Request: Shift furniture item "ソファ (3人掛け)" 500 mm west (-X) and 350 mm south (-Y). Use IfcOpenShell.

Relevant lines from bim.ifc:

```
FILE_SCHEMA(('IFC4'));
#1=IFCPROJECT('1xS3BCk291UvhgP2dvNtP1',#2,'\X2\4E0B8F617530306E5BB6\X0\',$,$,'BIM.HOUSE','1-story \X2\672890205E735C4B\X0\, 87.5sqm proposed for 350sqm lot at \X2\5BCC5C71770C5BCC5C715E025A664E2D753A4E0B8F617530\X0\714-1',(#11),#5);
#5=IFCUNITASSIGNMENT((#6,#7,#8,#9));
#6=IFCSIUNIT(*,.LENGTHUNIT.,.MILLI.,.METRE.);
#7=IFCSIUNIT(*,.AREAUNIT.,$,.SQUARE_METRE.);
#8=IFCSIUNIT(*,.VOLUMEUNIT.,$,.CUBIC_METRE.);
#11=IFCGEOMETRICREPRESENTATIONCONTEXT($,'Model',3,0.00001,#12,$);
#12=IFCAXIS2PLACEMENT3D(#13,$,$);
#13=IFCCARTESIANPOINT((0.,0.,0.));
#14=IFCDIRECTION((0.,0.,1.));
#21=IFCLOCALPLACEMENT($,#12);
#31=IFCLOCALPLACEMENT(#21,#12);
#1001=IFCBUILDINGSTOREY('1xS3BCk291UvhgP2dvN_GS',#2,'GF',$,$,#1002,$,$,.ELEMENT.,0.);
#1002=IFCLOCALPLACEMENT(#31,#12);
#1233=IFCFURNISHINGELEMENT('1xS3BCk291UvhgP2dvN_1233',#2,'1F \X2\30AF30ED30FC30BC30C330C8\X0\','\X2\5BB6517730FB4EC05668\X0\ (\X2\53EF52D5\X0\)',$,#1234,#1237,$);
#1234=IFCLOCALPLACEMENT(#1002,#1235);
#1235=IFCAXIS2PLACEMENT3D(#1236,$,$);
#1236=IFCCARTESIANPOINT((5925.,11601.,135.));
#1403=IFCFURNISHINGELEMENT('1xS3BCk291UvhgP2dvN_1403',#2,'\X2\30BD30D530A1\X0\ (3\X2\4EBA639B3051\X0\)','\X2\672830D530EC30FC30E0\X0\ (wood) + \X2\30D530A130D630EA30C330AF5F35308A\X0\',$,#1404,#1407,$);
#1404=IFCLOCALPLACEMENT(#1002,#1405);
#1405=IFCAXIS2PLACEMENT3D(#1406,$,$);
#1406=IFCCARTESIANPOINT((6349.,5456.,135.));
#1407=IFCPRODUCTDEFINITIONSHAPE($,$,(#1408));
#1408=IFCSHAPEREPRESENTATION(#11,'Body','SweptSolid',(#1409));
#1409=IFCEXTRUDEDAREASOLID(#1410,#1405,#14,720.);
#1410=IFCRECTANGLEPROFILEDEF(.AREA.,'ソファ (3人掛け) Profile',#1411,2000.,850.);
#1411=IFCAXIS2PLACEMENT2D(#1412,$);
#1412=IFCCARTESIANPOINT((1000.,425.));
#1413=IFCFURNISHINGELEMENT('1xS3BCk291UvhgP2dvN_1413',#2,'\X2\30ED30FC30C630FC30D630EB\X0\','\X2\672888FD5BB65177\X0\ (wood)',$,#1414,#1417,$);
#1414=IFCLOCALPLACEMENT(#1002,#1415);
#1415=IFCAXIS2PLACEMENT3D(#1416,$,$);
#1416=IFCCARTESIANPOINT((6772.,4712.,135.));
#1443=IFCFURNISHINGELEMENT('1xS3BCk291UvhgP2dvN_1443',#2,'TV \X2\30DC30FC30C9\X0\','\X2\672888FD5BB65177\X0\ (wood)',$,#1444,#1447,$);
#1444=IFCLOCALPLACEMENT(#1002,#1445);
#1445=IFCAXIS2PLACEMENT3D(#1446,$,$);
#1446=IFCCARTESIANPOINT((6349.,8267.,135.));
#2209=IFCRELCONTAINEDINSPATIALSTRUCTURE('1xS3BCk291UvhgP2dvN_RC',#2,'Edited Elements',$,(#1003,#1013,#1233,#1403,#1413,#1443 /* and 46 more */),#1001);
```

```python
import ifcopenshell
import ifcopenshell.api.geometry
import ifcopenshell.util.placement
import ifcopenshell.util.unit

model = ifcopenshell.open("bim.ifc")
unit_scale = ifcopenshell.util.unit.calculate_unit_scale(model)

item = model.by_id(1403)
matrix = ifcopenshell.util.placement.get_local_placement(item.ObjectPlacement)
matrix[0, 3] -= 0.5 / unit_scale
matrix[1, 3] -= 0.35 / unit_scale
ifcopenshell.api.geometry.edit_object_placement(model, product=item, matrix=matrix, is_si=False)

print(ifcopenshell.util.placement.get_local_placement(item.ObjectPlacement).round(3) + 0.0)

model.write("bim_v2.ifc")
```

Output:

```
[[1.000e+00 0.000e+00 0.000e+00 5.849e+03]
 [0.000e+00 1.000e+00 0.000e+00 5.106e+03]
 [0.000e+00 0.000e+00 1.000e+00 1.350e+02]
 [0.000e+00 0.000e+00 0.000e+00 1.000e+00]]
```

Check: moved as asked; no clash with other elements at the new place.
